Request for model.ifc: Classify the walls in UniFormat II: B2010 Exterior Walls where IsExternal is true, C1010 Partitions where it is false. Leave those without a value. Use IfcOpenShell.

First a look at what the model holds.

```python
import ifcopenshell
import ifcopenshell.util.element

model = ifcopenshell.open("model.ifc")
print(model.schema)
print("classifications:", [c.Name for c in model.by_type("IfcClassification")])
values = [ifcopenshell.util.element.get_pset(e, "Pset_WallCommon", "IsExternal") for e in model.by_type("IfcWall")]
for value in (True, False, None):
    print("IsExternal", value, values.count(value))
```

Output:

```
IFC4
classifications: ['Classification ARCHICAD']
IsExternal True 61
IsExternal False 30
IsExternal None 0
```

```python
import ifcopenshell
import ifcopenshell.api.classification
import ifcopenshell.util.element

model = ifcopenshell.open("model.ifc")

system = ifcopenshell.api.classification.add_classification(model, classification="UniFormat II")

walls = model.by_type("IfcWall")
external = {e: ifcopenshell.util.element.get_pset(e, "Pset_WallCommon", "IsExternal") for e in walls}
for flag, code, name in ((True, "B2010", "Exterior Walls"), (False, "C1010", "Partitions")):
    products = [e for e in walls if external[e] is flag]
    ifcopenshell.api.classification.add_reference(
        model, products=products, classification=system, identification=code, name=name
    )
    print(code, len(products))

model.write("model_rev.ifc")
```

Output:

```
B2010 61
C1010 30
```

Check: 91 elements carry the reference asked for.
